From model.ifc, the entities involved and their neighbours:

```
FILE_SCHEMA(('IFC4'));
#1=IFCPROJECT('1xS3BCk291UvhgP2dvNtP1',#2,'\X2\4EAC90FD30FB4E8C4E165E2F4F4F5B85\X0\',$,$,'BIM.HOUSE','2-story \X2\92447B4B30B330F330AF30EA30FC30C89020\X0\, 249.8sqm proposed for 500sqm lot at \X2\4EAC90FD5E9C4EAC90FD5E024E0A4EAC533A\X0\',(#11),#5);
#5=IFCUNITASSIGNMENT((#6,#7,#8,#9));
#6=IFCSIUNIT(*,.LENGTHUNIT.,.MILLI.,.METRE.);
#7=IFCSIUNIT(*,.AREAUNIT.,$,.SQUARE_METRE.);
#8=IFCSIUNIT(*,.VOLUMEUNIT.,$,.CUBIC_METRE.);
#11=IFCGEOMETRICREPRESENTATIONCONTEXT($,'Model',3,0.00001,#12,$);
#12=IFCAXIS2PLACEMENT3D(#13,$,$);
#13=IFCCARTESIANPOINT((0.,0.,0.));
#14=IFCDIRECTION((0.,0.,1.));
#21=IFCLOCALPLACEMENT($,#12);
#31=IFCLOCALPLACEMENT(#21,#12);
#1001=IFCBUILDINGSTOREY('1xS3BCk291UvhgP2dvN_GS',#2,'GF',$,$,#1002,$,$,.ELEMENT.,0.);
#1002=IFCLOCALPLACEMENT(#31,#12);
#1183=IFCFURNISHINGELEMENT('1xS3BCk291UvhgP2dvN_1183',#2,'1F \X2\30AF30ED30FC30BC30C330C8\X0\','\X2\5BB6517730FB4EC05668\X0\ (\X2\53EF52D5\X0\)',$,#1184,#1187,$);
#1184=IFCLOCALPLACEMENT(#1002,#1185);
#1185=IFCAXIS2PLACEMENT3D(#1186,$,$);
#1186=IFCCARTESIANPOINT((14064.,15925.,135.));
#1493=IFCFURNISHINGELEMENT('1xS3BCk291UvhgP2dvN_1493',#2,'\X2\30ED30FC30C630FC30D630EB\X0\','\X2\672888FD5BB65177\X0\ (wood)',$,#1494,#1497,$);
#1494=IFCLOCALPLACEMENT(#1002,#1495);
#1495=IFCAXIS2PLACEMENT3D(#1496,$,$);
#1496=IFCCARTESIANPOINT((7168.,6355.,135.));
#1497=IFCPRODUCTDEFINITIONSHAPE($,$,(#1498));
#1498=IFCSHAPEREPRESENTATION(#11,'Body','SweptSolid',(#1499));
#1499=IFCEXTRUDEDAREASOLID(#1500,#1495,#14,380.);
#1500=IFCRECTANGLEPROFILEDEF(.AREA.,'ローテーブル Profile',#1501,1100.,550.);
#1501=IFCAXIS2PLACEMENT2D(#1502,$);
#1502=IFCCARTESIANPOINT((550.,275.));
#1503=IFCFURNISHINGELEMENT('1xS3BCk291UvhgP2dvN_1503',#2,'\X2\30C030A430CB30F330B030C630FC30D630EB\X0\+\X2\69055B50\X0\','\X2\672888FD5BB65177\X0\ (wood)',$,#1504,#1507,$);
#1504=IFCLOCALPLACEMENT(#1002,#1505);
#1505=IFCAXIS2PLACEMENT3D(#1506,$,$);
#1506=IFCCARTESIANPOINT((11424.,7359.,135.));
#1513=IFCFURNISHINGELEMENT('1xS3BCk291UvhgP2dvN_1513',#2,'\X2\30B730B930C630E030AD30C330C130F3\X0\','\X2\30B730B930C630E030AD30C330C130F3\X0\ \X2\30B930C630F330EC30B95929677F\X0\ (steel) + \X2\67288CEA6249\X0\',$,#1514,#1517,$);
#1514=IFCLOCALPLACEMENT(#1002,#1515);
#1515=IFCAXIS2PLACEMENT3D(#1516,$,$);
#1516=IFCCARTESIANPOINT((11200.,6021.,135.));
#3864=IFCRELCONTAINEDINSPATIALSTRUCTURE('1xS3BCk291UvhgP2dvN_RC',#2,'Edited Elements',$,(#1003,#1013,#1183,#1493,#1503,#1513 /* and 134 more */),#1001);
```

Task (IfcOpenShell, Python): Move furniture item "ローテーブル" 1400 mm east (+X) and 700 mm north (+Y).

```python
import ifcopenshell
import ifcopenshell.api.geometry
import ifcopenshell.util.placement
import ifcopenshell.util.unit

model = ifcopenshell.open("model.ifc")
unit_scale = ifcopenshell.util.unit.calculate_unit_scale(model)

item = model.by_id(1493)
matrix = ifcopenshell.util.placement.get_local_placement(item.ObjectPlacement)
matrix[0, 3] += 1.4 / unit_scale
matrix[1, 3] += 0.7 / unit_scale
ifcopenshell.api.geometry.edit_object_placement(model, product=item, matrix=matrix, is_si=False)

print(ifcopenshell.util.placement.get_local_placement(item.ObjectPlacement).round(3) + 0.0)

model.write("model_v2.ifc")
```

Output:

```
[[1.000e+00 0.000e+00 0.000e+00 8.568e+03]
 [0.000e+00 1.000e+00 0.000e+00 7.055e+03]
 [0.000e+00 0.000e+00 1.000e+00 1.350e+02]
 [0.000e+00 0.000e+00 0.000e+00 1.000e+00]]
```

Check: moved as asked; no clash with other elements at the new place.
